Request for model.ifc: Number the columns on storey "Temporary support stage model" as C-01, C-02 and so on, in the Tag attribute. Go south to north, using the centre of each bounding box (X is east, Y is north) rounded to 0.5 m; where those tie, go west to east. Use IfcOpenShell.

First a look at what the model holds.

```python
import ifcopenshell
import ifcopenshell.util.element
import ifcopenshell.util.placement

model = ifcopenshell.open("model.ifc")
print(model.schema)
storey = next(s for s in model.by_type("IfcBuildingStorey") if s.Name == "Temporary support stage model")
columns = [e for e in ifcopenshell.util.element.get_decomposition(storey) if e.is_a("IfcColumn")]
for e in sorted(columns, key=lambda e: e.id()):
    origin = ifcopenshell.util.placement.get_local_placement(e.ObjectPlacement)[:3, 3]
    print(e.id(), e.Tag, e.Name, origin.round(2) + 0.0, sep=" | ")
```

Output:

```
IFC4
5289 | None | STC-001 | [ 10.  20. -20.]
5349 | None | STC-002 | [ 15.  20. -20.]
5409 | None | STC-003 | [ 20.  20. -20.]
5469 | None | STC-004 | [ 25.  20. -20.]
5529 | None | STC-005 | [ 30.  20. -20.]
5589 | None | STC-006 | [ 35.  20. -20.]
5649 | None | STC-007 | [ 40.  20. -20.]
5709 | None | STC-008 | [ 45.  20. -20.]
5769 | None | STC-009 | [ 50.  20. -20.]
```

```python
import ifcopenshell
import ifcopenshell.geom
import ifcopenshell.util.element
import ifcopenshell.util.shape

model = ifcopenshell.open("model.ifc")
settings = ifcopenshell.geom.settings()
settings.set("use-world-coords", True)


def centre(element):
    shape = ifcopenshell.geom.create_shape(settings, element)
    return ifcopenshell.util.shape.get_bbox_centroid(shape.geometry)


storey = next(s for s in model.by_type("IfcBuildingStorey") if s.Name == "Temporary support stage model")
columns = [e for e in ifcopenshell.util.element.get_decomposition(storey) if e.is_a("IfcColumn")]

# Insertion points can sit at a corner or the storey origin, so sort by the geometry (in metres).
centres = {e: centre(e) for e in columns}
columns.sort(key=lambda e: (round(centres[e][1] / 0.5), centres[e][0]))

for i, e in enumerate(columns, start=1):
    number = f"C-{i:02d}"
    e.Tag = number
    print(e.id(), number)

model.write("model_rev.ifc")
```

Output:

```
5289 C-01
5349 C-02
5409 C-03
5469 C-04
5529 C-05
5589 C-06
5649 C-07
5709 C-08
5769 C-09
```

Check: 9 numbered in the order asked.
